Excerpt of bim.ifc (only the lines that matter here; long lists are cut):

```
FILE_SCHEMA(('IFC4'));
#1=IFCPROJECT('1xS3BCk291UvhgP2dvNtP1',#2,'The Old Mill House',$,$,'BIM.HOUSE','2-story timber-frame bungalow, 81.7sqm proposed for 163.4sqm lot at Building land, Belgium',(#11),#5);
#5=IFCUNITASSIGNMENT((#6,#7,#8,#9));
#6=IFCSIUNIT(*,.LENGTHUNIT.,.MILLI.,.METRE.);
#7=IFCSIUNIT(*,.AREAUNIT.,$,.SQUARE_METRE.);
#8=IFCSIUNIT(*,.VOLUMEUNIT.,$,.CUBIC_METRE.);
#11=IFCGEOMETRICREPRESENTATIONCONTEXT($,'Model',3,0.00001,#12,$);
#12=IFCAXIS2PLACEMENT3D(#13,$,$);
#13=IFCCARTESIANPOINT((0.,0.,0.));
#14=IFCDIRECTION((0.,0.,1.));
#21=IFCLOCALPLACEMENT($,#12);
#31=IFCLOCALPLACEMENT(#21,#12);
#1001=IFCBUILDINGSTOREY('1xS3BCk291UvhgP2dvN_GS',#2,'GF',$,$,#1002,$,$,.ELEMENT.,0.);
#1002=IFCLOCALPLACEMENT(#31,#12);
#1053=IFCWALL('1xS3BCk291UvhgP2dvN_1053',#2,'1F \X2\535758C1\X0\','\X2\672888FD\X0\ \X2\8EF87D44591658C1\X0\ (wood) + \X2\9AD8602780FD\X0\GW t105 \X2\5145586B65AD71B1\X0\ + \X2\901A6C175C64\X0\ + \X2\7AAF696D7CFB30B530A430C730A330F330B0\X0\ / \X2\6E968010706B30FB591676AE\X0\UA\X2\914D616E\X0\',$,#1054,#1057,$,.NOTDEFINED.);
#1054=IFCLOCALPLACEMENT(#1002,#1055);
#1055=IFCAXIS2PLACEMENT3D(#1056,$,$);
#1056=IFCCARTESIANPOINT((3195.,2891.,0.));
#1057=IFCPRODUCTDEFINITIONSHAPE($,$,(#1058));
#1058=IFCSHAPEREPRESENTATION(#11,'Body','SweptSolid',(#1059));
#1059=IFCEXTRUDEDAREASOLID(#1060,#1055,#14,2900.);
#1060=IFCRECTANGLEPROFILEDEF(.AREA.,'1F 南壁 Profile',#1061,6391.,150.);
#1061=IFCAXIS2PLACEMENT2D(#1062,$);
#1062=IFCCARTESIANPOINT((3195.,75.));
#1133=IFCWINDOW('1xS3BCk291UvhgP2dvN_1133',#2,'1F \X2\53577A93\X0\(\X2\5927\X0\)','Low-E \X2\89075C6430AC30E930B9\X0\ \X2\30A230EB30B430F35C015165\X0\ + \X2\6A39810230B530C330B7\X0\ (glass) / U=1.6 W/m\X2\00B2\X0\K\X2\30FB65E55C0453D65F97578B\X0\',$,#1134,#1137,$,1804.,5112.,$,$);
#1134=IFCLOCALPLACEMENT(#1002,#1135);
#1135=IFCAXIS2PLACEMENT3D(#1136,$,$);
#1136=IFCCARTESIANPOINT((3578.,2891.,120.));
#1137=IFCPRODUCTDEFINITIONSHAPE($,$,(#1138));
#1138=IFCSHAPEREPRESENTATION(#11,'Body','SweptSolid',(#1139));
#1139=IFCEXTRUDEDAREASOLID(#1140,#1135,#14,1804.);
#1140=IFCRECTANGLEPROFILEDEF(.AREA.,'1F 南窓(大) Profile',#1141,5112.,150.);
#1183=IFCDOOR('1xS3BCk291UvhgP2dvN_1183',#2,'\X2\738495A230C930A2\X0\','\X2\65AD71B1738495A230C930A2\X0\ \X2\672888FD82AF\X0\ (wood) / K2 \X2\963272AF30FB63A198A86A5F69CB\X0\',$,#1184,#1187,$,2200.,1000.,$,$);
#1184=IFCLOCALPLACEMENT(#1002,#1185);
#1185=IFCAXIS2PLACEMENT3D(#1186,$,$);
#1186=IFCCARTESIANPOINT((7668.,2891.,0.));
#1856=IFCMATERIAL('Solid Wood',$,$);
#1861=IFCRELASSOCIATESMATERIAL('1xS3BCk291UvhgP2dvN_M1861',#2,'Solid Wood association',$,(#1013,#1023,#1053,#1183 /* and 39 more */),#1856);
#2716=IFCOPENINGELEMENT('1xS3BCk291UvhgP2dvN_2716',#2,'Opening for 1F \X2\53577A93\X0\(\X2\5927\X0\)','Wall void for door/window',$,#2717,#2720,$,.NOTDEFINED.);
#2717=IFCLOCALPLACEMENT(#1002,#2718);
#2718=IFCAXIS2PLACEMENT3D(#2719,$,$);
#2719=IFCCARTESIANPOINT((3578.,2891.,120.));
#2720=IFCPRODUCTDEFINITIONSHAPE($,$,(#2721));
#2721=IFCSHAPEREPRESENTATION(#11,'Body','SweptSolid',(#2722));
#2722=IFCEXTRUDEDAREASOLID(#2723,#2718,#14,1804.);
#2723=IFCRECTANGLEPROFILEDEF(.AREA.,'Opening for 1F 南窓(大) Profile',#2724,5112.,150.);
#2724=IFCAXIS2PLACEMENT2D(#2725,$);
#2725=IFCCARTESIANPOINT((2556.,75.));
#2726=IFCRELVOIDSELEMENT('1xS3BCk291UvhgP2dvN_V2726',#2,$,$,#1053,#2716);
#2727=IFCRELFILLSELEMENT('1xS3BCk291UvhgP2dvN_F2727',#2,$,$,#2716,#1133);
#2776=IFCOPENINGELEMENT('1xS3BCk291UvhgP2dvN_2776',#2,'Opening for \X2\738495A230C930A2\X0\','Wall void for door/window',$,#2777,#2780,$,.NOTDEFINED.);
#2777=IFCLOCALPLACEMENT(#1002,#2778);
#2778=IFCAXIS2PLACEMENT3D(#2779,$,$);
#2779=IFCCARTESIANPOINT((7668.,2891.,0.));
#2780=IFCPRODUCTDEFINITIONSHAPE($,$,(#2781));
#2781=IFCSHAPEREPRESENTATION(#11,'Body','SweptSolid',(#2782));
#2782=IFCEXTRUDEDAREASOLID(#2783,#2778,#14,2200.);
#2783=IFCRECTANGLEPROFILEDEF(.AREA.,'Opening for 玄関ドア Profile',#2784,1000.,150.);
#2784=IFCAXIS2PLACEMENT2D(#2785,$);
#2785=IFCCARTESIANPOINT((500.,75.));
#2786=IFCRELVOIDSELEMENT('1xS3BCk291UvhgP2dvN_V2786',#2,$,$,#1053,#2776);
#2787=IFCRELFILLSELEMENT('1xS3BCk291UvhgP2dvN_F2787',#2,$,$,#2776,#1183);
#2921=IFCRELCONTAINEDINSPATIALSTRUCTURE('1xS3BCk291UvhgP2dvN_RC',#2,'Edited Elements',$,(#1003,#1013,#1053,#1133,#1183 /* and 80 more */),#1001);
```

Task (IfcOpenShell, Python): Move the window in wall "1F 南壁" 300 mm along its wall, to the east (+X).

```python
import ifcopenshell
import ifcopenshell.api.geometry
import ifcopenshell.util.placement

model = ifcopenshell.open("bim.ifc")

window = model.by_guid("1xS3BCk291UvhgP2dvN_1133")
opening = window.FillsVoids[0].RelatingOpeningElement
wall = opening.VoidsElements[0].RelatingBuildingElement

wall_matrix = ifcopenshell.util.placement.get_local_placement(wall.ObjectPlacement)
shift = wall_matrix[:3, 0] * 300.0
before = ifcopenshell.util.placement.get_local_placement(window.ObjectPlacement)[:3, 3].copy()

# The window is not placed relative to its opening, so move both.
for product in (opening, window):
    matrix = ifcopenshell.util.placement.get_local_placement(product.ObjectPlacement)
    matrix[:3, 3] += shift
    ifcopenshell.api.geometry.edit_object_placement(model, product=product, matrix=matrix, is_si=False)

after = ifcopenshell.util.placement.get_local_placement(window.ObjectPlacement)[:3, 3]
print("window moved by", (after - before).round(3) + 0.0)

model.write("bim-out.ifc")
```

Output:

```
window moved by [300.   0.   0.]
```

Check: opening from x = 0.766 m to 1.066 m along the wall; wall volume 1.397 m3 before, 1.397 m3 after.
